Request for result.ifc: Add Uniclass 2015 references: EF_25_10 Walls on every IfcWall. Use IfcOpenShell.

First a look at what the model holds.

```python
import ifcopenshell

model = ifcopenshell.open("result.ifc")
print(model.schema)
print("classifications:", [c.Name for c in model.by_type("IfcClassification")])
for ifc_class in ("IfcDoor", "IfcRoof", "IfcStair", "IfcWall", "IfcWindow"):
    print(ifc_class, len(model.by_type(ifc_class)))
```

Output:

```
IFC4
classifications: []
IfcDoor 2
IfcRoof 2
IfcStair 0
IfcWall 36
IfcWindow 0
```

```python
import ifcopenshell
import ifcopenshell.api.classification

model = ifcopenshell.open("result.ifc")

system = ifcopenshell.api.classification.add_classification(model, classification="Uniclass 2015")

codes = {
    "IfcWall": ("EF_25_10", "Walls"),
}
for ifc_class, (code, name) in codes.items():
    products = model.by_type(ifc_class)
    ifcopenshell.api.classification.add_reference(
        model, products=products, classification=system, identification=code, name=name
    )
    print(code, len(products))

model.write("result_v2.ifc")
```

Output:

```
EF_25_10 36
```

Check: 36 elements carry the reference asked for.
